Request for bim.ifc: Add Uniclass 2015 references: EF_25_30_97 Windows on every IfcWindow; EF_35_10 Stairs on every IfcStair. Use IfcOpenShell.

First a look at what the model holds.

```python
import ifcopenshell

model = ifcopenshell.open("bim.ifc")
print(model.schema)
print("classifications:", [c.Name for c in model.by_type("IfcClassification")])
for ifc_class in ("IfcDoor", "IfcRoof", "IfcStair", "IfcWall", "IfcWindow"):
    print(ifc_class, len(model.by_type(ifc_class)))
```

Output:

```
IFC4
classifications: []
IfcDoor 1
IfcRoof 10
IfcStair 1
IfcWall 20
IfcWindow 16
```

```python
import ifcopenshell
import ifcopenshell.api.classification

model = ifcopenshell.open("bim.ifc")

system = ifcopenshell.api.classification.add_classification(model, classification="Uniclass 2015")

codes = {
    "IfcWindow": ("EF_25_30_97", "Windows"),
    "IfcStair": ("EF_35_10", "Stairs"),
}
for ifc_class, (code, name) in codes.items():
    products = model.by_type(ifc_class)
    ifcopenshell.api.classification.add_reference(
        model, products=products, classification=system, identification=code, name=name
    )
    print(code, len(products))

model.write("bim_updated.ifc")
```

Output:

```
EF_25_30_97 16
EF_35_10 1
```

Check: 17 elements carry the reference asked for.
